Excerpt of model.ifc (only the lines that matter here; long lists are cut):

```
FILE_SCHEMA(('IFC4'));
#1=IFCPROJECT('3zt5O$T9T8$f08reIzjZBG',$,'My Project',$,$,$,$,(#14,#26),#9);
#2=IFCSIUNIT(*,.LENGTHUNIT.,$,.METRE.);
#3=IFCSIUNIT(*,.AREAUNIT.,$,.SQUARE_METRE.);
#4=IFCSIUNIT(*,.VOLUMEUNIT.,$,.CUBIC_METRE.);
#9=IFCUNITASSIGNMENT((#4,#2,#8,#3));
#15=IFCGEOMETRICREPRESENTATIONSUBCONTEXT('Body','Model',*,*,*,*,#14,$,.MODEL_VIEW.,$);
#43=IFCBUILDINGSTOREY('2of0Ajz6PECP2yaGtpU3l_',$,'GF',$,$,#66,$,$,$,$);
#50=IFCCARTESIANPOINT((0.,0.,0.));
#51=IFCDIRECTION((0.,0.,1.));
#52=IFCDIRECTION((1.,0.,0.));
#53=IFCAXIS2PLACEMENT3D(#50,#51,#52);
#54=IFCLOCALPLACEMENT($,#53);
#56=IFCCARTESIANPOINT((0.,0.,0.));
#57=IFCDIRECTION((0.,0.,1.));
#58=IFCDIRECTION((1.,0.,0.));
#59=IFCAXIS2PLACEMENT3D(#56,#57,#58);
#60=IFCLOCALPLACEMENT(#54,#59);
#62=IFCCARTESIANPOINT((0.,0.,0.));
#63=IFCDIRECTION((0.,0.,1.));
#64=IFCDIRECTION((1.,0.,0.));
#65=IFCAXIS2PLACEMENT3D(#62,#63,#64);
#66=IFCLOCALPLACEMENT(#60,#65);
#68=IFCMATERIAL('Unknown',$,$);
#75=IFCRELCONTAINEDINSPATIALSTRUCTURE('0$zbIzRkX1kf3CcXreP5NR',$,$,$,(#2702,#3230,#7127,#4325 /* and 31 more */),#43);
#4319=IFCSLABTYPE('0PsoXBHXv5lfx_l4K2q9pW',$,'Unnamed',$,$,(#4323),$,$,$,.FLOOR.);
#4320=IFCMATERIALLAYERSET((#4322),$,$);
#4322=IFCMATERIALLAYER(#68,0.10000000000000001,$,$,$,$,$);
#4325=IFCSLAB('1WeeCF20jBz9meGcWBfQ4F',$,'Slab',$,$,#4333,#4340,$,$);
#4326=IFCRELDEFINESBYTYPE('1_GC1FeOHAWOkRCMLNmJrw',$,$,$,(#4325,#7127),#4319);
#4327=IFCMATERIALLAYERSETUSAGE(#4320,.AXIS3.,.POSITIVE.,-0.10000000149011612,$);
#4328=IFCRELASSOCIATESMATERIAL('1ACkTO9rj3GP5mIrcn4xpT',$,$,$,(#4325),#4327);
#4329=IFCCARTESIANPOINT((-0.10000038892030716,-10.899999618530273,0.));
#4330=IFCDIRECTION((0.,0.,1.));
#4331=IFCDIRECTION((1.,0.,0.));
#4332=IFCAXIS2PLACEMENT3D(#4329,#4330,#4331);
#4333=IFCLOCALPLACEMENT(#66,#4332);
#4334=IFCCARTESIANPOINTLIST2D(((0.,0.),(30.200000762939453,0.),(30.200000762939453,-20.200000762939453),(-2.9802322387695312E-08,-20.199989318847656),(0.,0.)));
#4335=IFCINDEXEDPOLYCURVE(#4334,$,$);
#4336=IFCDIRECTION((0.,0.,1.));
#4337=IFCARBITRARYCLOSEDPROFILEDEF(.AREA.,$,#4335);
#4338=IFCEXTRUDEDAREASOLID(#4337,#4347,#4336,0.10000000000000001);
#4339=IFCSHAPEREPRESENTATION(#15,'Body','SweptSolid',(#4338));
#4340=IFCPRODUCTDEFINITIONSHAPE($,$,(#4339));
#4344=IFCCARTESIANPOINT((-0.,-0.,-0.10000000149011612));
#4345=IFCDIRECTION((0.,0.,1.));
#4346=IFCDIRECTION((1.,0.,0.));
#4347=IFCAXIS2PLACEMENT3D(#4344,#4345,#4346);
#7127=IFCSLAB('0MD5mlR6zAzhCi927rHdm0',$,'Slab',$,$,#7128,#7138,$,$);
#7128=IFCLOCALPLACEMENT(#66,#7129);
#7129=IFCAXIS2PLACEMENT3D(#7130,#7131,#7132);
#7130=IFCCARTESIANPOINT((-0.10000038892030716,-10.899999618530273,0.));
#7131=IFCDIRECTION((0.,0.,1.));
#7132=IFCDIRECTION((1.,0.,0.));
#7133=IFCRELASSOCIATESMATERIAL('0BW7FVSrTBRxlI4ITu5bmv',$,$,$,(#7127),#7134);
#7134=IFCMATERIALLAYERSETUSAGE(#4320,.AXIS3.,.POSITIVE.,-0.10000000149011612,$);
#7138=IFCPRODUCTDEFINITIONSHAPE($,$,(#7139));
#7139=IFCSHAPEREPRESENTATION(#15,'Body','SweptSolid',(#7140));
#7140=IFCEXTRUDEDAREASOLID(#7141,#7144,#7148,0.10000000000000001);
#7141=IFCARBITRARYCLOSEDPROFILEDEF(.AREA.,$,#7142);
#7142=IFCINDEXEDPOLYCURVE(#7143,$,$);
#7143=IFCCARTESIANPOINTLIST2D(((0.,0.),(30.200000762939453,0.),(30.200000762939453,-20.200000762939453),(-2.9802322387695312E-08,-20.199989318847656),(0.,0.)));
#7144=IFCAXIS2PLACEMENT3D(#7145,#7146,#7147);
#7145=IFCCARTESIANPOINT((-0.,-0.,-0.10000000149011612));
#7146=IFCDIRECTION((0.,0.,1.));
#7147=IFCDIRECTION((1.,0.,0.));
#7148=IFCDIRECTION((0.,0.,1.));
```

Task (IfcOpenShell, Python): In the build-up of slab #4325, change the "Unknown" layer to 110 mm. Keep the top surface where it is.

```python
import ifcopenshell
import ifcopenshell.util.element
import ifcopenshell.util.representation

model = ifcopenshell.open("model.ifc")

layer_set = model.by_id(4320)
layer = next(l for l in layer_set.MaterialLayers if l.Material and l.Material.Name == "Unknown")
change = 0.11 - layer.LayerThickness
layer.LayerThickness += change

# The layer set is shared, so every slab that uses it gets the new thickness.
slabs = [e for e in ifcopenshell.util.element.get_elements_by_material(model, layer_set) if e.is_a("IfcSlab")]
for slab in sorted(slabs, key=lambda e: e.id()):
    body = ifcopenshell.util.representation.get_representation(slab, "Model", "Body")
    solid = body.Items[0]
    old_depth = solid.Depth
    solid.Depth += change
    # Extruded upwards: lower the start of the extrusion so the top stays.
    x, y, z = solid.Position.Location.Coordinates
    solid.Position.Location = model.createIfcCartesianPoint((x, y, z - change))
    print(slab.id(), f"{old_depth:g} -> {solid.Depth:g}")

# The layers are counted up from the underside, which has moved.
for usage in {ifcopenshell.util.element.get_material(slab) for slab in slabs}:
    usage.OffsetFromReferenceLine -= change

model.write("model-out.ifc")
```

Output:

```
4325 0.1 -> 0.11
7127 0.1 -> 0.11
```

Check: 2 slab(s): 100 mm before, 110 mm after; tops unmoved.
